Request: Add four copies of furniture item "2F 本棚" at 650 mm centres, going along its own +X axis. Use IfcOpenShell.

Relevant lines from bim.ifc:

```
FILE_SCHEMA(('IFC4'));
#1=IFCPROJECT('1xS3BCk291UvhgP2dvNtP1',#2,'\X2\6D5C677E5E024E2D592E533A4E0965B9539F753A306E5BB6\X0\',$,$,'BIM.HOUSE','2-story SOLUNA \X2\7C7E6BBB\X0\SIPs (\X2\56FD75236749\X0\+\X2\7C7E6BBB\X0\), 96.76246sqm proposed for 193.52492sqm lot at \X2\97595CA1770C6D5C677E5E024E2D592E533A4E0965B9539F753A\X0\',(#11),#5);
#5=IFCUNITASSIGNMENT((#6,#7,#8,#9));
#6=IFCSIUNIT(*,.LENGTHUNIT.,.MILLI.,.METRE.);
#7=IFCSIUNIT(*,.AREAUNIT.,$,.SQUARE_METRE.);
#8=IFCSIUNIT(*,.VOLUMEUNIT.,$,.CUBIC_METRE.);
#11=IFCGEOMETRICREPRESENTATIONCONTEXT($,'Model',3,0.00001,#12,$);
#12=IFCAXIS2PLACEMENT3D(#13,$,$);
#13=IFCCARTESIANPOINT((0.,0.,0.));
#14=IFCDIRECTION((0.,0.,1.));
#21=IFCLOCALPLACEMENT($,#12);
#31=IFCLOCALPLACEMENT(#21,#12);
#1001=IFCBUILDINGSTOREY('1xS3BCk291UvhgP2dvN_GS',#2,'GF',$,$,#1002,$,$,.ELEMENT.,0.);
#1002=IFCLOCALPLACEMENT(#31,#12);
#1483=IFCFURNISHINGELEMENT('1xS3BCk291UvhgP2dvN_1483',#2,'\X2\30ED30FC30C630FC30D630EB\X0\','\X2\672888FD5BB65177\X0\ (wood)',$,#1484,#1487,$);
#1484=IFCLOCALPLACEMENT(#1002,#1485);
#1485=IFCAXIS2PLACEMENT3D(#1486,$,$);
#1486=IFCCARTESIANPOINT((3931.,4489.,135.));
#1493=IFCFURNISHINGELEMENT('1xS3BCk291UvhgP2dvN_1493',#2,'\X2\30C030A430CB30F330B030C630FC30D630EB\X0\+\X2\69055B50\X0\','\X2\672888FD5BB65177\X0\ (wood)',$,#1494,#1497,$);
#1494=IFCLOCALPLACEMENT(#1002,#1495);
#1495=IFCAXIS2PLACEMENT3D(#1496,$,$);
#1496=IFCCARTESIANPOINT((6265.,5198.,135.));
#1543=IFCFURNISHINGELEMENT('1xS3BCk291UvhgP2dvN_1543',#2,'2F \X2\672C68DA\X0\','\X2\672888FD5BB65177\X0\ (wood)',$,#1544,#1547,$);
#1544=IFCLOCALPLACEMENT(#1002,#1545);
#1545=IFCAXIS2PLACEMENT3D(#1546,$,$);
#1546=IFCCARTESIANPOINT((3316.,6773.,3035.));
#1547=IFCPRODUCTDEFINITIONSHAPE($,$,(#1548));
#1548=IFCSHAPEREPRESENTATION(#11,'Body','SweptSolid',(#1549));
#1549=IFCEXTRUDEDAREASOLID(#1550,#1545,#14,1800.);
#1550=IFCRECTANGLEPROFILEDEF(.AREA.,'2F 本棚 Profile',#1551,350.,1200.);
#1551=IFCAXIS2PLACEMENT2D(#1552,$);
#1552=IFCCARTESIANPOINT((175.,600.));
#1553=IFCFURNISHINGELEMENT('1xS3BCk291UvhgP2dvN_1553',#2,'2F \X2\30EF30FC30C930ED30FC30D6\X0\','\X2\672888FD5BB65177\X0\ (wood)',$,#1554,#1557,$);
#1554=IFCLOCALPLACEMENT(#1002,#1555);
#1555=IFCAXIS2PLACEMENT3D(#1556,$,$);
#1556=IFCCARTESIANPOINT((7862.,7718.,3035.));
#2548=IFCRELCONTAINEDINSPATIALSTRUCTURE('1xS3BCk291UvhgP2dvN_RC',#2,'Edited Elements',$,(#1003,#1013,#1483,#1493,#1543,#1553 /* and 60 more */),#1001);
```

```python
import ifcopenshell
import ifcopenshell.api.geometry
import ifcopenshell.api.root
import ifcopenshell.util.element
import ifcopenshell.util.placement
import ifcopenshell.util.unit

model = ifcopenshell.open("bim.ifc")
unit_scale = ifcopenshell.util.unit.calculate_unit_scale(model)


def reuse_history(source, copy):
    """copy_class also copies each property set's owner history, people and application; keep the originals."""
    for rel in copy.IsDefinedBy:
        if rel.is_a("IfcRelDefinesByProperties") and (history := rel.RelatingPropertyDefinition.OwnerHistory):
            rel.RelatingPropertyDefinition.OwnerHistory = source.OwnerHistory
            ifcopenshell.util.element.remove_deep2(model, history)


source = model.by_guid("1xS3BCk291UvhgP2dvN_1543")
base = ifcopenshell.util.placement.get_local_placement(source.ObjectPlacement)
step = base[:3, 0] * 0.65 / unit_scale

for i in range(1, 5):
    copy = ifcopenshell.api.root.copy_class(model, product=source)
    copy.Representation = ifcopenshell.util.element.copy_deep(
        model, source.Representation, exclude=["IfcGeometricRepresentationContext", "IfcRepresentationMap"]
    )
    reuse_history(source, copy)
    matrix = base.copy()
    matrix[:3, 3] += i * step
    print("added at", matrix[:3, 3].round(3) + 0.0)
    ifcopenshell.api.geometry.edit_object_placement(model, product=copy, matrix=matrix, is_si=False)

model.write("bim_edited.ifc")
```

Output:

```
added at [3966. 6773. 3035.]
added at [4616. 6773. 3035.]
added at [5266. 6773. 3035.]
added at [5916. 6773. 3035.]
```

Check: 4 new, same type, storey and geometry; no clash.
